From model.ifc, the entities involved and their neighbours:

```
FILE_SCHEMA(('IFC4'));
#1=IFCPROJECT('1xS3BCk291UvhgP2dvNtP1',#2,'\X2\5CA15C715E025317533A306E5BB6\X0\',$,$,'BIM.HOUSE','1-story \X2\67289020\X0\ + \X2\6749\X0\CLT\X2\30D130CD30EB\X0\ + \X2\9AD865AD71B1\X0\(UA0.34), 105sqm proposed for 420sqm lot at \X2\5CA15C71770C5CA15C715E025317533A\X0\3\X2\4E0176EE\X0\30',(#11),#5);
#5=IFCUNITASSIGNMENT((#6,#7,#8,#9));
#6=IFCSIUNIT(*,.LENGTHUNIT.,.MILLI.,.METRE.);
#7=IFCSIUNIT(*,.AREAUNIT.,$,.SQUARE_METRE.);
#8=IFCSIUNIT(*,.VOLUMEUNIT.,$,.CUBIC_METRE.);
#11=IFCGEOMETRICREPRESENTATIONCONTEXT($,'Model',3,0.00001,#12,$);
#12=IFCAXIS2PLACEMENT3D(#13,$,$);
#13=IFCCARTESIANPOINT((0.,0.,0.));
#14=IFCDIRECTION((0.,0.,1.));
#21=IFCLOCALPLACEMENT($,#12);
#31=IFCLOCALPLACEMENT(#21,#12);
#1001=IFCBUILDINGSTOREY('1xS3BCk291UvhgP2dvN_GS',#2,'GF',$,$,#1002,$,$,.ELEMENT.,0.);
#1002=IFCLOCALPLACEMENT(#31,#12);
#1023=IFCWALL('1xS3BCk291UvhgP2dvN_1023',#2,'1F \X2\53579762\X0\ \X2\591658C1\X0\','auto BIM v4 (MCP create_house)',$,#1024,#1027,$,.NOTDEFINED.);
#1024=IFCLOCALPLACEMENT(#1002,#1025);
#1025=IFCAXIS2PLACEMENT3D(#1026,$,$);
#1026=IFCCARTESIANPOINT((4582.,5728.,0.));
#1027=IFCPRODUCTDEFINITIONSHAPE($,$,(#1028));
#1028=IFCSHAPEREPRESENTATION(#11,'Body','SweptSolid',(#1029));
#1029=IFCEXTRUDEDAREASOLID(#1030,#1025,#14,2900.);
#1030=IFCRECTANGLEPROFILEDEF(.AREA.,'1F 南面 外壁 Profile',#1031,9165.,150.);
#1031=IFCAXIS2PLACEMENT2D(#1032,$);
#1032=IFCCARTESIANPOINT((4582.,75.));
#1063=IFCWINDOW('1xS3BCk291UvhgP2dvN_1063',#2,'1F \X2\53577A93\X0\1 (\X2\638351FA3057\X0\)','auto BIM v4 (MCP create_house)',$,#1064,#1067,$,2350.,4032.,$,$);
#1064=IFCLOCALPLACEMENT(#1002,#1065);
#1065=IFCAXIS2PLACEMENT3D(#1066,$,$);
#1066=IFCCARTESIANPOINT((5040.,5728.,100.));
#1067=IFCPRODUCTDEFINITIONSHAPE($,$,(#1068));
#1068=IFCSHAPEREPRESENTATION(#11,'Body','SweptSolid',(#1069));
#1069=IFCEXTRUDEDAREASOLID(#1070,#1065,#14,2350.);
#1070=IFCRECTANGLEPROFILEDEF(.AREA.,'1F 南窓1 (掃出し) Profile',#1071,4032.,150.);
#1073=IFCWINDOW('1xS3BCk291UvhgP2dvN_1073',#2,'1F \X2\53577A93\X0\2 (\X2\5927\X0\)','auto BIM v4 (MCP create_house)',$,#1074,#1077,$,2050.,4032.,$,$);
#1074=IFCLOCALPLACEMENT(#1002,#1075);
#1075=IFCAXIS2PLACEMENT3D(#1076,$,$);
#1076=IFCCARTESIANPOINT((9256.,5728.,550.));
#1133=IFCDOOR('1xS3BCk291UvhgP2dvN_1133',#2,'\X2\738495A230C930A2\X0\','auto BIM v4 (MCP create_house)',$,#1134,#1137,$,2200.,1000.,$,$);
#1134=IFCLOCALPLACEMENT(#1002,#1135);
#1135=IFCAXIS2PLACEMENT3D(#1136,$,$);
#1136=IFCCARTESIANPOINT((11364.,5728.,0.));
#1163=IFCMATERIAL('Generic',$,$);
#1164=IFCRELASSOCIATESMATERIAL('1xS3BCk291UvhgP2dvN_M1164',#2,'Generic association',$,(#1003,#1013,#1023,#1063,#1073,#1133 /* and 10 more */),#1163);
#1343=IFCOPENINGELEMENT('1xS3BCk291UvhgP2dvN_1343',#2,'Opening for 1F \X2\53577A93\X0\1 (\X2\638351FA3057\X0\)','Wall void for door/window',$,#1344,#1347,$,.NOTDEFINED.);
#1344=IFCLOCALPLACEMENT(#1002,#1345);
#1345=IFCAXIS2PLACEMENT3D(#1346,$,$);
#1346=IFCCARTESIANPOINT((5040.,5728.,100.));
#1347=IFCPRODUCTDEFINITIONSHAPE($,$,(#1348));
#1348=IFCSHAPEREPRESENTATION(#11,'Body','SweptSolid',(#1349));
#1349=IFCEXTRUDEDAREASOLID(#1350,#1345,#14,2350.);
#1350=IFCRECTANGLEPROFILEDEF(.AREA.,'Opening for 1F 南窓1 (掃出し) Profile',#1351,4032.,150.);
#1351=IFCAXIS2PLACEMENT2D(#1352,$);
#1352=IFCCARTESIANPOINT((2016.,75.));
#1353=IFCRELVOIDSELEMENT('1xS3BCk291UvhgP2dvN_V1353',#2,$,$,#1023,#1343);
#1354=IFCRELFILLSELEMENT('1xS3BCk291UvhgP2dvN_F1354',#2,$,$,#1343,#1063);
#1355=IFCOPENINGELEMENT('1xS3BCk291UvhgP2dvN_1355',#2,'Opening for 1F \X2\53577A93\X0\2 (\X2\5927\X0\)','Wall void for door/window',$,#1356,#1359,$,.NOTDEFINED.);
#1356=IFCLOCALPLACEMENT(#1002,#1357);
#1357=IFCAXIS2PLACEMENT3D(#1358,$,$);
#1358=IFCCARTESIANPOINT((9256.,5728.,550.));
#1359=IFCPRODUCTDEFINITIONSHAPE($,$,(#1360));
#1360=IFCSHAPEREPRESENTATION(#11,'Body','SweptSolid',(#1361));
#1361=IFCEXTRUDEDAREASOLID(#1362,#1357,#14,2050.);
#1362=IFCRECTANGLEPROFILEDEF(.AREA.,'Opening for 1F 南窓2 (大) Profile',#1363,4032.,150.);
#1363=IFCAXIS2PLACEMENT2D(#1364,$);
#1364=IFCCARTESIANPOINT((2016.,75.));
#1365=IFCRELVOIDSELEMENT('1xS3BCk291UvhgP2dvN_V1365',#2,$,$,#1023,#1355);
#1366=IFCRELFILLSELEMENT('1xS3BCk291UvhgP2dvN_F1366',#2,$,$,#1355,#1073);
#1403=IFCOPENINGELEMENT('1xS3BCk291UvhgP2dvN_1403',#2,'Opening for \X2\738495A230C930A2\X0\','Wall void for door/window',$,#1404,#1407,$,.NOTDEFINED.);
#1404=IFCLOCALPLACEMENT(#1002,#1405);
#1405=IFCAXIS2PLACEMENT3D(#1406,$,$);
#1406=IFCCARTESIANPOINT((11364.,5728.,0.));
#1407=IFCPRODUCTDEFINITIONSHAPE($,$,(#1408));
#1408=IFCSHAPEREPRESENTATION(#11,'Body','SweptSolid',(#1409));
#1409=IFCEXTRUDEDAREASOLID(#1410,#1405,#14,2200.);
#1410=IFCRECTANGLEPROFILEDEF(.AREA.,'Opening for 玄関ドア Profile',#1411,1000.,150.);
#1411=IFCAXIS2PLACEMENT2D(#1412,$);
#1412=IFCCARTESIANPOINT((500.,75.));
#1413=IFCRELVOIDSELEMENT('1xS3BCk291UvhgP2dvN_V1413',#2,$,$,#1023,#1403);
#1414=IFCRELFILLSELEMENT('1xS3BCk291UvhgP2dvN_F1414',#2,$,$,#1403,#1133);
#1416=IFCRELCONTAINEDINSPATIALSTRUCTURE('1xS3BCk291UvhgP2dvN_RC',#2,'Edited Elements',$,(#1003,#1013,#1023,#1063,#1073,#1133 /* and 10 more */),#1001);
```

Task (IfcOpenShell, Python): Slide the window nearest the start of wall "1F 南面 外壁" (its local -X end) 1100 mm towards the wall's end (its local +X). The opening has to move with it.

```python
import ifcopenshell
import ifcopenshell.api.geometry
import ifcopenshell.util.placement
import ifcopenshell.util.unit

model = ifcopenshell.open("model.ifc")
unit_scale = ifcopenshell.util.unit.calculate_unit_scale(model)

window = model.by_guid("1xS3BCk291UvhgP2dvN_1063")
opening = window.FillsVoids[0].RelatingOpeningElement
wall = opening.VoidsElements[0].RelatingBuildingElement

wall_matrix = ifcopenshell.util.placement.get_local_placement(wall.ObjectPlacement)
shift = wall_matrix[:3, 0] * 1.1 / unit_scale
before = ifcopenshell.util.placement.get_local_placement(window.ObjectPlacement)[:3, 3].copy()

# The window is not placed relative to its opening, so move both.
for product in (opening, window):
    matrix = ifcopenshell.util.placement.get_local_placement(product.ObjectPlacement)
    matrix[:3, 3] += shift
    ifcopenshell.api.geometry.edit_object_placement(model, product=product, matrix=matrix, is_si=False)

after = ifcopenshell.util.placement.get_local_placement(window.ObjectPlacement)[:3, 3]
print("window moved by", (after - before).round(3) + 0.0)

model.write("model_v2.ifc")
```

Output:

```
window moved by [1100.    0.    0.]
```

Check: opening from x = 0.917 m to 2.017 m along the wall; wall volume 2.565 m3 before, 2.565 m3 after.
